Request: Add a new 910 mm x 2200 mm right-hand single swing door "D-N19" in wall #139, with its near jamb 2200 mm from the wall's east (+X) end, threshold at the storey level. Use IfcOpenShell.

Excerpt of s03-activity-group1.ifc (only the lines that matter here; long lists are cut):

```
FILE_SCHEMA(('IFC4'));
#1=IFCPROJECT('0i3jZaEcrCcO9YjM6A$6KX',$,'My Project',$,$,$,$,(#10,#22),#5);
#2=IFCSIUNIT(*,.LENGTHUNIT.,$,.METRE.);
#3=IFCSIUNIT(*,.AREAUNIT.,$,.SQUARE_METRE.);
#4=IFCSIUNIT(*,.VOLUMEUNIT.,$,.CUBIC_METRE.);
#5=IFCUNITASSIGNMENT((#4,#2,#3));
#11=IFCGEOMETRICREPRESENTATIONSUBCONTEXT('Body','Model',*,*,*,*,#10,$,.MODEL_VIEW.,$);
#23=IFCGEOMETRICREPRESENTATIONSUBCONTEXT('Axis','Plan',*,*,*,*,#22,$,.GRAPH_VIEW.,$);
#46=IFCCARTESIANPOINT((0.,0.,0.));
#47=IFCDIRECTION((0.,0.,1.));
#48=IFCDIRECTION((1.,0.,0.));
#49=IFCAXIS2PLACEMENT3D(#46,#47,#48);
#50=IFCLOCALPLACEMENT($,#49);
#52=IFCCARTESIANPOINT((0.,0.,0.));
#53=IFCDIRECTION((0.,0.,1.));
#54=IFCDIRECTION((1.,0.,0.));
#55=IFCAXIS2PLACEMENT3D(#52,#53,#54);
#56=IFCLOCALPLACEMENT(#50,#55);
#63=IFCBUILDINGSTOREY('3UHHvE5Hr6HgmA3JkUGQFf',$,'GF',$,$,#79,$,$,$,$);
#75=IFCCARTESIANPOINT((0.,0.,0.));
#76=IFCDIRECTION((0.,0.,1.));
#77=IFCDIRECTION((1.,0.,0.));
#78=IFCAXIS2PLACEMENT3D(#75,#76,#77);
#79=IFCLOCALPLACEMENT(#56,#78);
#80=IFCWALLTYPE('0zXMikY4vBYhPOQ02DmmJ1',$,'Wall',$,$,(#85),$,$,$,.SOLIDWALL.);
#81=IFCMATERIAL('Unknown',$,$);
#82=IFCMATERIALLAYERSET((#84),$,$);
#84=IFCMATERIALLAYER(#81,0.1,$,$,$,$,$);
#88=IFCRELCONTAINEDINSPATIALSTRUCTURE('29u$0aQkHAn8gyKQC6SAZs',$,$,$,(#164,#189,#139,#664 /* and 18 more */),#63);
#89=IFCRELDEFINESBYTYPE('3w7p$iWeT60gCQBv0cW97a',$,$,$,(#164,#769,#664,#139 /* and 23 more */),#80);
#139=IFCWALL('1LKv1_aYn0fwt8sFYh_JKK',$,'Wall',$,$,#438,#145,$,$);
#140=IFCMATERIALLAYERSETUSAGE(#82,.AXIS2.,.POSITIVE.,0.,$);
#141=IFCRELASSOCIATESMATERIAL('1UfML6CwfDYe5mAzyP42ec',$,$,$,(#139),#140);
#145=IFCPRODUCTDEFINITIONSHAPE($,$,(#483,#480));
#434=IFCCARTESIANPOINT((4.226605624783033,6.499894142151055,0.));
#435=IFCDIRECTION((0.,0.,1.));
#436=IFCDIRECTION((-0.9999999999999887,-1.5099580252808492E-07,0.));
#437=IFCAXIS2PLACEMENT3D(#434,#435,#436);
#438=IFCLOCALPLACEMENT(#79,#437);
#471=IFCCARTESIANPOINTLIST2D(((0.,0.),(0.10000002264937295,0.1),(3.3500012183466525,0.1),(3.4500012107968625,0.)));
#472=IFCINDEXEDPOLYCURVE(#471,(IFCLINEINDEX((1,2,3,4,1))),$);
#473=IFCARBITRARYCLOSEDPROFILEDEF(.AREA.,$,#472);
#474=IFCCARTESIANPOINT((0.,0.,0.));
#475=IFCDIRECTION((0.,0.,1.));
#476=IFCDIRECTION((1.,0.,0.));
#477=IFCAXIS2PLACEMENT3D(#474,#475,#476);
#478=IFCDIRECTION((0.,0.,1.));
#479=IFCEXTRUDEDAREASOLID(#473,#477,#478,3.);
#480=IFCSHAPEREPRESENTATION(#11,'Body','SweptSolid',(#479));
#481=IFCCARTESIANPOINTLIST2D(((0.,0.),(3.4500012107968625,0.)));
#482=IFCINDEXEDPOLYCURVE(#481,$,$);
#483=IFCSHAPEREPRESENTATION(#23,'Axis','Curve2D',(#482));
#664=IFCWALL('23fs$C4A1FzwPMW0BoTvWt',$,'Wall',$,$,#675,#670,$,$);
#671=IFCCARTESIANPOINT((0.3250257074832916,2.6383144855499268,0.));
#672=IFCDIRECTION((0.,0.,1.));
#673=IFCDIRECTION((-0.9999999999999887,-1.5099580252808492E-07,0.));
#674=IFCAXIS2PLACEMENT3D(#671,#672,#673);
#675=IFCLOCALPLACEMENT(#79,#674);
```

```python
import numpy as np
import ifcopenshell
import ifcopenshell.api.feature
import ifcopenshell.api.geometry
import ifcopenshell.api.root
import ifcopenshell.api.spatial
import ifcopenshell.geom
import ifcopenshell.util.element
import ifcopenshell.util.placement
import ifcopenshell.util.representation
import ifcopenshell.util.shape
import ifcopenshell.util.unit

model = ifcopenshell.open("s03-activity-group1.ifc")
unit_scale = ifcopenshell.util.unit.calculate_unit_scale(model)
settings = ifcopenshell.geom.settings()


def volume(element):
    """Net volume in cubic metres, openings subtracted."""
    shape = ifcopenshell.geom.create_shape(settings, element)
    return ifcopenshell.util.shape.get_volume(shape.geometry)


wall = model.by_guid("1LKv1_aYn0fwt8sFYh_JKK")
storey = ifcopenshell.util.element.get_container(wall, ifc_class="IfcBuildingStorey")
context = ifcopenshell.util.representation.get_context(model, "Model", "Body", "MODEL_VIEW")
before = volume(wall)

width, height, from_end, sill = 0.91, 2.2, 2.2, 0.0  # metres

# The wall runs along its own X axis, and the end named is its -X end.
wall_shape = ifcopenshell.geom.create_shape(settings, wall)
x, y, z = ifcopenshell.util.shape.get_vertices(wall_shape.geometry).T
start = x.min() + from_end
face, thickness = float(y.min()), float(y.max() - y.min())
wall_matrix = ifcopenshell.util.placement.get_local_placement(wall.ObjectPlacement)
level = ifcopenshell.util.placement.get_local_placement(storey.ObjectPlacement)[2, 3]


def in_wall(x, y):
    """Placement at x, y metres in the wall's axes, at sill height."""
    matrix = wall_matrix.copy()
    matrix[:, 3] = wall_matrix @ np.array([x / unit_scale, y / unit_scale, 0.0, 1.0])
    matrix[2, 3] = level + sill / unit_scale
    return matrix


# Opening: a box that overshoots both wall faces by 50 mm.
opening = ifcopenshell.api.root.create_entity(model, ifc_class="IfcOpeningElement", predefined_type="OPENING")
box = ifcopenshell.api.geometry.add_wall_representation(
    model, context=context, length=width, height=height, thickness=thickness + 0.1
)
ifcopenshell.api.geometry.assign_representation(model, product=opening, representation=box)
ifcopenshell.api.geometry.edit_object_placement(model, product=opening, matrix=in_wall(start, face - 0.05), is_si=False)
ifcopenshell.api.feature.add_feature(model, feature=opening, element=wall)

door = ifcopenshell.api.root.create_entity(model, ifc_class="IfcDoor", name="D-N19", predefined_type="DOOR")
door.OverallWidth, door.OverallHeight = width / unit_scale, height / unit_scale
door.OperationType = "SINGLE_SWING_RIGHT"
body = ifcopenshell.api.geometry.add_door_representation(
    model,
    context=context,
    overall_width=door.OverallWidth,
    overall_height=door.OverallHeight,
    operation_type="SINGLE_SWING_RIGHT",
    lining_properties={"LiningDepth": thickness / unit_scale, "ThresholdDepth": thickness / unit_scale},
)
ifcopenshell.api.geometry.assign_representation(model, product=door, representation=body)
ifcopenshell.api.spatial.assign_container(model, products=[door], relating_structure=storey)
ifcopenshell.api.feature.add_filling(model, opening=opening, element=door)

# The lining spans the wall, so the door starts at the wall face.
ifcopenshell.api.geometry.edit_object_placement(model, product=door, matrix=in_wall(start, face), is_si=False)

after = volume(wall)

print(f"wall volume {before:.3f} -> {after:.3f} m3")

model.write("s03-activity-group1_v2.ifc")
```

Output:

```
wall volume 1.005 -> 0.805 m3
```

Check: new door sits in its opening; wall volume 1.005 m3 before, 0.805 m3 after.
